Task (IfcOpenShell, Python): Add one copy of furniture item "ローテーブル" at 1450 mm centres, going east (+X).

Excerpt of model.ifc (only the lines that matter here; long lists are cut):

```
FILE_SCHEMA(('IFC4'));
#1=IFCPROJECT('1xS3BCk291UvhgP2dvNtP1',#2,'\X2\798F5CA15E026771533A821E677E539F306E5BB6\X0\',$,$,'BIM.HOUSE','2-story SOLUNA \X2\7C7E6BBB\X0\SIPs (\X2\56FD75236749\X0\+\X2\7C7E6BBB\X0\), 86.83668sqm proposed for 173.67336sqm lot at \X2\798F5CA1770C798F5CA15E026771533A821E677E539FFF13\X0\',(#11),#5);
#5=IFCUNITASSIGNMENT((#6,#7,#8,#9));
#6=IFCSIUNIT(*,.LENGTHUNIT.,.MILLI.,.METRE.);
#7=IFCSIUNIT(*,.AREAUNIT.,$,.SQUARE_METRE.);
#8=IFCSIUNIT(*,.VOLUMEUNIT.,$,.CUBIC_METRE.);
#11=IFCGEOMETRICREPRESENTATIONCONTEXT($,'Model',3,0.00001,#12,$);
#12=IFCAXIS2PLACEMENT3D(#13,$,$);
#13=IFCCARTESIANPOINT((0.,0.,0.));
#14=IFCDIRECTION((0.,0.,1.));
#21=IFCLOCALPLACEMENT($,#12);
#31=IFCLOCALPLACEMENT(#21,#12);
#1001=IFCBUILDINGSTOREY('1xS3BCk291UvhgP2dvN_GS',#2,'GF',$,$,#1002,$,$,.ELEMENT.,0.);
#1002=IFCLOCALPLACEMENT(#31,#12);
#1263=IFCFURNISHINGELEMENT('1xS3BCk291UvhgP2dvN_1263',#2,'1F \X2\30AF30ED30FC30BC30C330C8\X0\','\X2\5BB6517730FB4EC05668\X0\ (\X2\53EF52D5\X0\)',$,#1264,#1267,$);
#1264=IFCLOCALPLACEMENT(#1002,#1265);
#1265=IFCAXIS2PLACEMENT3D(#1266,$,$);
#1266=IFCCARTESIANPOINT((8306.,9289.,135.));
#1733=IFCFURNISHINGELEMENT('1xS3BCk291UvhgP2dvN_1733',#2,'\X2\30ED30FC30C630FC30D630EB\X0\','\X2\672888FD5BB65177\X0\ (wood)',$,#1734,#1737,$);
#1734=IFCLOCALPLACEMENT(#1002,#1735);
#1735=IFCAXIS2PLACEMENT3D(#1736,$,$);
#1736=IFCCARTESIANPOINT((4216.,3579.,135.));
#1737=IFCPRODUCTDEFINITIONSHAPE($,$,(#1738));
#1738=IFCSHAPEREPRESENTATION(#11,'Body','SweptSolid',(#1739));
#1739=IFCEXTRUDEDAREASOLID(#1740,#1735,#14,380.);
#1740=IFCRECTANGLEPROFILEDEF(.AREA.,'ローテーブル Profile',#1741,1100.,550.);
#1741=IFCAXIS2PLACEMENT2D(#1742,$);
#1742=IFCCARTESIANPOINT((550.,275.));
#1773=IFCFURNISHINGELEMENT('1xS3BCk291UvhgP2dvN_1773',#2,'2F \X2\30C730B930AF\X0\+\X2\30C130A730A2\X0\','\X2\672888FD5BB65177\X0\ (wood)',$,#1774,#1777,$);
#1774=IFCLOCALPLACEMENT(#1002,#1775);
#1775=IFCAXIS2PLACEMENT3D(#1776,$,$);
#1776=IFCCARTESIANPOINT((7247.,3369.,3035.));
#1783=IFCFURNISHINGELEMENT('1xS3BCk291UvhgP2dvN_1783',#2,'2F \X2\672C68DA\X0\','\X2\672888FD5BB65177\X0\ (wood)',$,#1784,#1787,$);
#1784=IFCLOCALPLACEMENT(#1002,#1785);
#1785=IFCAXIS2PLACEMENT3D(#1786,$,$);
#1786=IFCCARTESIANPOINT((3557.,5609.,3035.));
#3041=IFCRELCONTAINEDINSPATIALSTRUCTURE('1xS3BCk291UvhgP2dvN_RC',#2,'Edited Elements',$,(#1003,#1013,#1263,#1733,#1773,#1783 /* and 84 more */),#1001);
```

```python
import numpy as np
import ifcopenshell
import ifcopenshell.api.geometry
import ifcopenshell.api.root
import ifcopenshell.util.element
import ifcopenshell.util.placement

model = ifcopenshell.open("model.ifc")


def reuse_history(source, copy):
    """copy_class also copies each property set's owner history, people and application; keep the originals."""
    for rel in copy.IsDefinedBy:
        if rel.is_a("IfcRelDefinesByProperties") and (history := rel.RelatingPropertyDefinition.OwnerHistory):
            rel.RelatingPropertyDefinition.OwnerHistory = source.OwnerHistory
            ifcopenshell.util.element.remove_deep2(model, history)


source = model.by_guid("1xS3BCk291UvhgP2dvN_1733")
base = ifcopenshell.util.placement.get_local_placement(source.ObjectPlacement)
step = np.array([1.0, 0.0, 0.0]) * 1450.0

for i in range(1, 2):
    copy = ifcopenshell.api.root.copy_class(model, product=source)
    copy.Representation = ifcopenshell.util.element.copy_deep(
        model, source.Representation, exclude=["IfcGeometricRepresentationContext", "IfcRepresentationMap"]
    )
    reuse_history(source, copy)
    matrix = base.copy()
    matrix[:3, 3] += i * step
    print("added at", matrix[:3, 3].round(3) + 0.0)
    ifcopenshell.api.geometry.edit_object_placement(model, product=copy, matrix=matrix, is_si=False)

model.write("model_v2.ifc")
```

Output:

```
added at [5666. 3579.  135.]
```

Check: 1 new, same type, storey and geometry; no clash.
